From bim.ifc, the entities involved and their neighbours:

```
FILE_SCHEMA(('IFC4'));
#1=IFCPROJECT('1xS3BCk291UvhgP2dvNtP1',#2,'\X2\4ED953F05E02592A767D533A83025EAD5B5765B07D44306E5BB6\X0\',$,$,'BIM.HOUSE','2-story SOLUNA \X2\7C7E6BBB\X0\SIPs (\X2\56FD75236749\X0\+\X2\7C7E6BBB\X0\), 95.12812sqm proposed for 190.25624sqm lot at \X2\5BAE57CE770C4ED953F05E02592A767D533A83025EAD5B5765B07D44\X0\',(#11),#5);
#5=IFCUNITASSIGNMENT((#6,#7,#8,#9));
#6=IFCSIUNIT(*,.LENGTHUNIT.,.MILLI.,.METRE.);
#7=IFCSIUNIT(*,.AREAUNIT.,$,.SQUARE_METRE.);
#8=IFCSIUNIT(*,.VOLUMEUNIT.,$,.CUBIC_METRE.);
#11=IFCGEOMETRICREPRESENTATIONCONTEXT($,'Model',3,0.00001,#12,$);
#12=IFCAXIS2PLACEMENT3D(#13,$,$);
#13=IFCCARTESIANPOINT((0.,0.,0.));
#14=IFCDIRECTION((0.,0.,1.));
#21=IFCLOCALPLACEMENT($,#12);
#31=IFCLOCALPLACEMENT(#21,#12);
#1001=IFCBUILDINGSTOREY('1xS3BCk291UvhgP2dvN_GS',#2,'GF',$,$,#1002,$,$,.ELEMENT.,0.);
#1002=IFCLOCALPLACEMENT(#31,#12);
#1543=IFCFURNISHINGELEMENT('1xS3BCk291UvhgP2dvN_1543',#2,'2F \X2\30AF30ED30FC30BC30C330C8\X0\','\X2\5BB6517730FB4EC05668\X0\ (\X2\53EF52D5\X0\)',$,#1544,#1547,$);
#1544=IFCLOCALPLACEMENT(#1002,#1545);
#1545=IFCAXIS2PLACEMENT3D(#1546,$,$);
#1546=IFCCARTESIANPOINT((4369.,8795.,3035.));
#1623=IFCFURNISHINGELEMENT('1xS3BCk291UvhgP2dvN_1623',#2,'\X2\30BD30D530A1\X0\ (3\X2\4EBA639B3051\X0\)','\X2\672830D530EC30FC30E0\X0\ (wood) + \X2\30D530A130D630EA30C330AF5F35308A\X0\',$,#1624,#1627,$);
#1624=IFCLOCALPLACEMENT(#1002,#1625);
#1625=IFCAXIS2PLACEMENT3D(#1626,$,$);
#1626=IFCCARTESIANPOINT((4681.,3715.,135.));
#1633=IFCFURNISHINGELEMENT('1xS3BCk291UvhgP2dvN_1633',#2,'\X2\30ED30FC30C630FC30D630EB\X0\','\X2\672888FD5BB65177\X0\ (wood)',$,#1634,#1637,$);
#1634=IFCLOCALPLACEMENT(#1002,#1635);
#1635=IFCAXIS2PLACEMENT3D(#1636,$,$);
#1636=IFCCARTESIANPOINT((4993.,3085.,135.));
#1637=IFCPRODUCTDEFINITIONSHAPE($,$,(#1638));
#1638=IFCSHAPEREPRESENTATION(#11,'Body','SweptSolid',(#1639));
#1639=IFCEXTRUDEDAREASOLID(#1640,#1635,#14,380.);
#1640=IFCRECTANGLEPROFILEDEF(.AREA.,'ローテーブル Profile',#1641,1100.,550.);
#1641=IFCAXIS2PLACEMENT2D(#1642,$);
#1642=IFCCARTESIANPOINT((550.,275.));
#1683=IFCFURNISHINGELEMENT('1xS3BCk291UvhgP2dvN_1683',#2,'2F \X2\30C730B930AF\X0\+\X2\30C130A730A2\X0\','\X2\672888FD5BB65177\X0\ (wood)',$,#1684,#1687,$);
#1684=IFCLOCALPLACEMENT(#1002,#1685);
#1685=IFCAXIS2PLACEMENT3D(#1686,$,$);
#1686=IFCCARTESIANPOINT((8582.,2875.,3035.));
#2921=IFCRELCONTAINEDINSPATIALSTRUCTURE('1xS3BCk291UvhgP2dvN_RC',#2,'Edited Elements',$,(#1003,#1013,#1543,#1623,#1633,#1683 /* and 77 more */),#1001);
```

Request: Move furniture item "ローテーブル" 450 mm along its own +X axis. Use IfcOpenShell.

```python
import ifcopenshell
import ifcopenshell.api.geometry
import ifcopenshell.util.placement
import ifcopenshell.util.unit

model = ifcopenshell.open("bim.ifc")
unit_scale = ifcopenshell.util.unit.calculate_unit_scale(model)

item = model.by_guid("1xS3BCk291UvhgP2dvN_1633")
matrix = ifcopenshell.util.placement.get_local_placement(item.ObjectPlacement)
matrix[:3, 3] += matrix[:3, 0] * 0.45 / unit_scale
ifcopenshell.api.geometry.edit_object_placement(model, product=item, matrix=matrix, is_si=False)

print(ifcopenshell.util.placement.get_local_placement(item.ObjectPlacement).round(3) + 0.0)

model.write("bim_rev.ifc")
```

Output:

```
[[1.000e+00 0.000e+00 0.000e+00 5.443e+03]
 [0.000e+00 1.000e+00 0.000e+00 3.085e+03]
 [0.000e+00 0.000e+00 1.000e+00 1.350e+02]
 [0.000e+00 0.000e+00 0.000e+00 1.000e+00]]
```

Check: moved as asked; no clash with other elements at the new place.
